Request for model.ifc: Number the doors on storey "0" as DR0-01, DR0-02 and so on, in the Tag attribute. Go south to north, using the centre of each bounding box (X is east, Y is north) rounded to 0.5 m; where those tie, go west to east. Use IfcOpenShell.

First a look at what the model holds.

```python
import ifcopenshell
import ifcopenshell.util.element
import ifcopenshell.util.placement

model = ifcopenshell.open("model.ifc")
print(model.schema)
storey = next(s for s in model.by_type("IfcBuildingStorey") if s.Name == "0")
doors = [e for e in ifcopenshell.util.element.get_decomposition(storey) if e.is_a("IfcDoor")]
for e in sorted(doors, key=lambda e: e.id()):
    origin = ifcopenshell.util.placement.get_local_placement(e.ObjectPlacement)[:3, 3]
    print(e.id(), e.Tag, e.Name, origin.round(2) + 0.0, sep=" | ")
```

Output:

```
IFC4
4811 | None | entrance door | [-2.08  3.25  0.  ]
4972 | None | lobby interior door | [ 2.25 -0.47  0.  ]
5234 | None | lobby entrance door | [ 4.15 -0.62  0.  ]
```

```python
import ifcopenshell
import ifcopenshell.geom
import ifcopenshell.util.element
import ifcopenshell.util.shape

model = ifcopenshell.open("model.ifc")
settings = ifcopenshell.geom.settings()
settings.set("use-world-coords", True)


def centre(element):
    shape = ifcopenshell.geom.create_shape(settings, element)
    return ifcopenshell.util.shape.get_bbox_centroid(shape.geometry)


storey = next(s for s in model.by_type("IfcBuildingStorey") if s.Name == "0")
doors = [e for e in ifcopenshell.util.element.get_decomposition(storey) if e.is_a("IfcDoor")]

# Insertion points can sit at a corner or the storey origin, so sort by the geometry (in metres).
centres = {e: centre(e) for e in doors}
doors.sort(key=lambda e: (round(centres[e][1] / 0.5), centres[e][0]))

for i, e in enumerate(doors, start=1):
    number = f"DR0-{i:02d}"
    e.Tag = number
    print(e.id(), number)

model.write("model_updated.ifc")
```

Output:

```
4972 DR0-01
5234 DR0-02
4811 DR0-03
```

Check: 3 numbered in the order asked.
